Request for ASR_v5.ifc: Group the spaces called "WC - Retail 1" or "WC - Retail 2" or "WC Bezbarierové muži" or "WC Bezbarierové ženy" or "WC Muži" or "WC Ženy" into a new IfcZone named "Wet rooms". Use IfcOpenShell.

First a look at what the model holds.

```python
import ifcopenshell

model = ifcopenshell.open("ASR_v5.ifc")
print(model.schema)
seen = {}
for space in model.by_type("IfcSpace"):
    seen[space.LongName] = seen.get(space.LongName, 0) + 1
for name, count in sorted(seen.items(), key=str):
    print(count, "x", name)
print("zones:", [z.Name for z in model.by_type("IfcZone")][:20])
```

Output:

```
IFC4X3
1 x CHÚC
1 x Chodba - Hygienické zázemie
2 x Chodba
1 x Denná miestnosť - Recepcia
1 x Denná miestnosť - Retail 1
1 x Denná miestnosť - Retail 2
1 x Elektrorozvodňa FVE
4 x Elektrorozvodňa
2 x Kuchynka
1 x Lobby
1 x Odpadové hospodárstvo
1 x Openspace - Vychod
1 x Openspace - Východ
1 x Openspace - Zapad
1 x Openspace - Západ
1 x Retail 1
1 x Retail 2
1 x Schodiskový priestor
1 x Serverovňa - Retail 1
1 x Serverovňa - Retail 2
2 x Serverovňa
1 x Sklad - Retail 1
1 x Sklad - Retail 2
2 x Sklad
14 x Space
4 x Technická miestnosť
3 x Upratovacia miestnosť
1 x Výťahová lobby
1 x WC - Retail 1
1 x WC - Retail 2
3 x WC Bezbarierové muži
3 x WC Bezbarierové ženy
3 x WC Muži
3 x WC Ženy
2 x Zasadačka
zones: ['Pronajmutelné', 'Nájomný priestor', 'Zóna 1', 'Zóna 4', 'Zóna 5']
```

```python
import ifcopenshell
import ifcopenshell.api.group
import ifcopenshell.api.root

model = ifcopenshell.open("ASR_v5.ifc")

names = {"WC - Retail 1", "WC - Retail 2", "WC Bezbarierové muži", "WC Bezbarierové ženy", "WC Muži", "WC Ženy"}
spaces = [s for s in model.by_type("IfcSpace") if s.LongName in names]

zone = ifcopenshell.api.root.create_entity(model, ifc_class="IfcZone", name="Wet rooms")
ifcopenshell.api.group.assign_group(model, products=spaces, group=zone)
print(len(spaces), "spaces in", zone.Name)

model.write("ASR_v5_rev.ifc")
```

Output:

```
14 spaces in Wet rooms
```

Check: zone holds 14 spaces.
